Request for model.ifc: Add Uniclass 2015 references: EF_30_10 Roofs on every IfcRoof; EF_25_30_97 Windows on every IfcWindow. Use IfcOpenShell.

First a look at what the model holds.

```python
import ifcopenshell

model = ifcopenshell.open("model.ifc")
print(model.schema)
print("classifications:", [c.Name for c in model.by_type("IfcClassification")])
for ifc_class in ("IfcDoor", "IfcRoof", "IfcStair", "IfcWall", "IfcWindow"):
    print(ifc_class, len(model.by_type(ifc_class)))
```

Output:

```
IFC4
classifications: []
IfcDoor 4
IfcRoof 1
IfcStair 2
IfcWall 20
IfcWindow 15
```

```python
import ifcopenshell
import ifcopenshell.api.classification

model = ifcopenshell.open("model.ifc")

system = ifcopenshell.api.classification.add_classification(model, classification="Uniclass 2015")

codes = {
    "IfcRoof": ("EF_30_10", "Roofs"),
    "IfcWindow": ("EF_25_30_97", "Windows"),
}
for ifc_class, (code, name) in codes.items():
    products = model.by_type(ifc_class)
    ifcopenshell.api.classification.add_reference(
        model, products=products, classification=system, identification=code, name=name
    )
    print(code, len(products))

model.write("model_rev.ifc")
```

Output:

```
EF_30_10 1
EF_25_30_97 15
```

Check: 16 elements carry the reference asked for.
